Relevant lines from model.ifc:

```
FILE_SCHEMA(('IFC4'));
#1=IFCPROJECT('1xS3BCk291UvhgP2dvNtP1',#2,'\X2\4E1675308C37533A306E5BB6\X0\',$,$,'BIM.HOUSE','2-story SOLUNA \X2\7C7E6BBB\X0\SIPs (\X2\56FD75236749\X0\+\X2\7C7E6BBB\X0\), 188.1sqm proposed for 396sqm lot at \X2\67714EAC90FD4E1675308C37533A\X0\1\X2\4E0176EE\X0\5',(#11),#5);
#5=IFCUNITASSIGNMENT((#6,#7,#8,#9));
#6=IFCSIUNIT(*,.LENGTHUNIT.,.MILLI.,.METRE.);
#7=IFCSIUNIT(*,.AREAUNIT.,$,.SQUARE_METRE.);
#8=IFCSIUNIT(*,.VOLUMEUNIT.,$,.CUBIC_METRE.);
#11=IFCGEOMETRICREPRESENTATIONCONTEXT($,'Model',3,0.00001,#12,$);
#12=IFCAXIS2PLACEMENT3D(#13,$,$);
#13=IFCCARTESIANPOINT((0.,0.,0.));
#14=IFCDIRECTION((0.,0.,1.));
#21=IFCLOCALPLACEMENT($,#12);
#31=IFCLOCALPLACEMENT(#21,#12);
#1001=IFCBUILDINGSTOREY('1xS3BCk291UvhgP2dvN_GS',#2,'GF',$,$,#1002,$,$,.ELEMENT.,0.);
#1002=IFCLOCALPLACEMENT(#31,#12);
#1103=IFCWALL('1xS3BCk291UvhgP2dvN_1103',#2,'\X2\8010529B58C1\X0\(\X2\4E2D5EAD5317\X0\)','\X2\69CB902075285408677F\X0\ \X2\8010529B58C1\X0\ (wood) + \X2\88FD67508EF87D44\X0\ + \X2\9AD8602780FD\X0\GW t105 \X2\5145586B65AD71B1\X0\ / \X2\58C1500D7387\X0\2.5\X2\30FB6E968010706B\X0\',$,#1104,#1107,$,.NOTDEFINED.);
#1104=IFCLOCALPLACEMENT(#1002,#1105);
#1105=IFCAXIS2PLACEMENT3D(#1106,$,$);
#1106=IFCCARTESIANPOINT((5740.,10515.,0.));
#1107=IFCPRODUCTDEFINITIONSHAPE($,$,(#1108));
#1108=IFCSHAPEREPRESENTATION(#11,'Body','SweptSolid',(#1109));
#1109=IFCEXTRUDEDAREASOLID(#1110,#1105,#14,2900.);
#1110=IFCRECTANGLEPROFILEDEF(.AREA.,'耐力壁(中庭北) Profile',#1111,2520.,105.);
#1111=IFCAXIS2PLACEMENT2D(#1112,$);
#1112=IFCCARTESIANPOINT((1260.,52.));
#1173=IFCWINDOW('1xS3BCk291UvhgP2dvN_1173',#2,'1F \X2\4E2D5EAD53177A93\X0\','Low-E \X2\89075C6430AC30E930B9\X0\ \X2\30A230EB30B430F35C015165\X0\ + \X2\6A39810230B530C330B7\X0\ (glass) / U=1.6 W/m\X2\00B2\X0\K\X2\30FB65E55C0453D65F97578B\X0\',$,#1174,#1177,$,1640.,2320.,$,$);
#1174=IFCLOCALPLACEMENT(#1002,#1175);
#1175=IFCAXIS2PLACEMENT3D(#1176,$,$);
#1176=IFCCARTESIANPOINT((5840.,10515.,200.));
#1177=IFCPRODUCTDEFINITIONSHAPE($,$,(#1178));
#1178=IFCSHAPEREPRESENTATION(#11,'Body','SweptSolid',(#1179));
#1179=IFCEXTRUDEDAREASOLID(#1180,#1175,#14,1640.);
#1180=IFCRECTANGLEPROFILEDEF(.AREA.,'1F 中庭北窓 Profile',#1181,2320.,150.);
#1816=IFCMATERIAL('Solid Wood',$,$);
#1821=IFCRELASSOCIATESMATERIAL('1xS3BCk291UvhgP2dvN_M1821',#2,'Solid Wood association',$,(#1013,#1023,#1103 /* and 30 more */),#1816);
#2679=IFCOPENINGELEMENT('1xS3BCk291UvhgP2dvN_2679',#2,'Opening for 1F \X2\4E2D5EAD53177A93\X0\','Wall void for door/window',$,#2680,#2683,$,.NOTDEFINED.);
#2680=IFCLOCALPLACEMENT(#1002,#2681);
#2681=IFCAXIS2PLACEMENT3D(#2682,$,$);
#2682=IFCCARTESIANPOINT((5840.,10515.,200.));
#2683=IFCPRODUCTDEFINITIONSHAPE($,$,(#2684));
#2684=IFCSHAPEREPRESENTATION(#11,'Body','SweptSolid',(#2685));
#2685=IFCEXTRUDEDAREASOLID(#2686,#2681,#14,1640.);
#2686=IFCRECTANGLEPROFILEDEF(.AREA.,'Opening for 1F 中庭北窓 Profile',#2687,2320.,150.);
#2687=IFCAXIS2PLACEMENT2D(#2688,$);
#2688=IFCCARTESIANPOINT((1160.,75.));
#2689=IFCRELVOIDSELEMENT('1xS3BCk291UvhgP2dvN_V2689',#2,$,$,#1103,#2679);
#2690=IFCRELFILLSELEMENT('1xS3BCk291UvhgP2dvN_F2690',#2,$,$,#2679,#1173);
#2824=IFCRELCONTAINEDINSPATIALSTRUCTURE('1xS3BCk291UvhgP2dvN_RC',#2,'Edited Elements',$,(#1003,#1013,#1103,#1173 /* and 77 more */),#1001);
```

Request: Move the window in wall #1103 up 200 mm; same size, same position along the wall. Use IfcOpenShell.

```python
import numpy as np
import ifcopenshell
import ifcopenshell.api.geometry
import ifcopenshell.util.placement
import ifcopenshell.util.unit

model = ifcopenshell.open("model.ifc")
unit_scale = ifcopenshell.util.unit.calculate_unit_scale(model)

window = model.by_guid("1xS3BCk291UvhgP2dvN_1173")
opening = window.FillsVoids[0].RelatingOpeningElement
dz = 0.2 / unit_scale

shift = np.array([0.0, 0.0, dz])
# The window is not placed relative to its opening, so move both.
for product in (opening, window):
    matrix = ifcopenshell.util.placement.get_local_placement(product.ObjectPlacement)
    matrix[:3, 3] += shift
    ifcopenshell.api.geometry.edit_object_placement(model, product=product, matrix=matrix, is_si=False)

print(f"moved by {dz * unit_scale:+.3f} m")

model.write("model_v2.ifc")
```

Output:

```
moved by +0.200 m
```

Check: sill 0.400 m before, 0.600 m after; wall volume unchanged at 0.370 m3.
